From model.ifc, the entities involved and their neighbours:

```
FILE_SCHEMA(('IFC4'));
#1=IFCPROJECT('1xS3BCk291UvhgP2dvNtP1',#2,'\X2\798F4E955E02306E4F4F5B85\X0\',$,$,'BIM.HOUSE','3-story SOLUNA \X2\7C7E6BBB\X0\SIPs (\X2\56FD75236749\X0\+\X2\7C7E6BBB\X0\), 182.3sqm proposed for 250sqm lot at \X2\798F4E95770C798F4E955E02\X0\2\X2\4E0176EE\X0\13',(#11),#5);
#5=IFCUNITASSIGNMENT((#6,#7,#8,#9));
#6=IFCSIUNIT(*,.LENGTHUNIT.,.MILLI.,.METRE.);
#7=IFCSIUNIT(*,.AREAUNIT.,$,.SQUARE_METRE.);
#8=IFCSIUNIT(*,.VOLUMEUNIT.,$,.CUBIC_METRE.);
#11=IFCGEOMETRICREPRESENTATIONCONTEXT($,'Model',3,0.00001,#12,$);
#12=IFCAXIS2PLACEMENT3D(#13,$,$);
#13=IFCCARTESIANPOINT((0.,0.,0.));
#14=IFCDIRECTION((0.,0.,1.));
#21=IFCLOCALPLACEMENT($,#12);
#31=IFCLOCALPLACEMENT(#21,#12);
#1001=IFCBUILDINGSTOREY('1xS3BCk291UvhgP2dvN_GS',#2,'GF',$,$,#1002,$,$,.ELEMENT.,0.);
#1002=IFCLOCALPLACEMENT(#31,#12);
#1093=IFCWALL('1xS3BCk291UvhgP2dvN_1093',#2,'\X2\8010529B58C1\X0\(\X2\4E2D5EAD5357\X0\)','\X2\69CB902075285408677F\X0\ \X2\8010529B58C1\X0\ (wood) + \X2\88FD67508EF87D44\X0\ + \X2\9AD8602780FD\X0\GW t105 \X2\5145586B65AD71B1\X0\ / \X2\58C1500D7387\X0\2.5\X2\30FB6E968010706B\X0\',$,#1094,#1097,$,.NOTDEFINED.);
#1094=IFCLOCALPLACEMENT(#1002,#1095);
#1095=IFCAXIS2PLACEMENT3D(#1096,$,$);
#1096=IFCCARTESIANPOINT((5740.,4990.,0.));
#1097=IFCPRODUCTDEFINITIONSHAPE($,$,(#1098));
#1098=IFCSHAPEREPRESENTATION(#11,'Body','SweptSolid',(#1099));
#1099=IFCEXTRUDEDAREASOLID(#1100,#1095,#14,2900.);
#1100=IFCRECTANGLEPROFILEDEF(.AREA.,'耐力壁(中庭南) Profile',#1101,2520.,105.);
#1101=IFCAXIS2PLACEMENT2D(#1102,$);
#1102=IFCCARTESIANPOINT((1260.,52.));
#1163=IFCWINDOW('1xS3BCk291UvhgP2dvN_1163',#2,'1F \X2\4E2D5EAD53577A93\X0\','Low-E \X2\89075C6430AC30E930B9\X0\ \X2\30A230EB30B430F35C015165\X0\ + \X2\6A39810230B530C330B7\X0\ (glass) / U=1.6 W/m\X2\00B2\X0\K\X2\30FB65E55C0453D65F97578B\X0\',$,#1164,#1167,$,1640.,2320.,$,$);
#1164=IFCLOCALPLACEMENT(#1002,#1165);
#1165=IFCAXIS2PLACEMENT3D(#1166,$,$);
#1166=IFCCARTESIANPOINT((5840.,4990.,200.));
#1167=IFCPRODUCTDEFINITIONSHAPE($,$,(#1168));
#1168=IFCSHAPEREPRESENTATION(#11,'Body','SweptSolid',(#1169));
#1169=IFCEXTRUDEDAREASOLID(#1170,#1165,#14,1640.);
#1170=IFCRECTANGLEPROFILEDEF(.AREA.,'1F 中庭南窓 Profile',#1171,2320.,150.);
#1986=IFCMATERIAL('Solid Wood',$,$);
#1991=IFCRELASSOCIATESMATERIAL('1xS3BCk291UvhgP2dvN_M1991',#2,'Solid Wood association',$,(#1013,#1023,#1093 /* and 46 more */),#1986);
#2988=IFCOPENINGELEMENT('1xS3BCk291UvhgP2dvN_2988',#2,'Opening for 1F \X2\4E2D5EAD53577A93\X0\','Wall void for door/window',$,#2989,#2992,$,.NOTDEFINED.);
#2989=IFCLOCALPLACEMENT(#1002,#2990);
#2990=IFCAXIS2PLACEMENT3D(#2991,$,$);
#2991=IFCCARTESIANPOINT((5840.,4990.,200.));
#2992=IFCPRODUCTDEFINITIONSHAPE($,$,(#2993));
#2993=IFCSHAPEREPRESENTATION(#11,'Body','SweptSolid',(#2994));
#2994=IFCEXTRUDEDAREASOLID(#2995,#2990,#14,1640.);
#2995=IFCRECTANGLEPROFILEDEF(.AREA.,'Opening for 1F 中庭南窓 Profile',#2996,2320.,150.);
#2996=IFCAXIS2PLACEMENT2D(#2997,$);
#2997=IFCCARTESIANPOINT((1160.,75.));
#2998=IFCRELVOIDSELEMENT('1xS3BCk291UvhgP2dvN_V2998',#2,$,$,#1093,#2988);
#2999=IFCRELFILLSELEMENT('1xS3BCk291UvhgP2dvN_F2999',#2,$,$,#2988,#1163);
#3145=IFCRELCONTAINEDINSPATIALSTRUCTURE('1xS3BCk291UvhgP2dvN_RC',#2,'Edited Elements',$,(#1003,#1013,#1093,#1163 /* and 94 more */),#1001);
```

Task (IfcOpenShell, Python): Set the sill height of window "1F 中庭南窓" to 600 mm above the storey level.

```python
import numpy as np
import ifcopenshell
import ifcopenshell.api.geometry
import ifcopenshell.geom
import ifcopenshell.util.element
import ifcopenshell.util.placement
import ifcopenshell.util.shape
import ifcopenshell.util.unit

model = ifcopenshell.open("model.ifc")
unit_scale = ifcopenshell.util.unit.calculate_unit_scale(model)

window = model.by_id(1163)
opening = window.FillsVoids[0].RelatingOpeningElement
storey = ifcopenshell.util.element.get_container(window, ifc_class="IfcBuildingStorey")
level = ifcopenshell.util.placement.get_local_placement(storey.ObjectPlacement)[2, 3]

# The opening's origin need not be at the sill, so measure its lowest point.
shape = ifcopenshell.geom.create_shape(ifcopenshell.geom.settings(), opening)
bottom = ifcopenshell.util.shape.get_shape_bottom_elevation(shape, shape.geometry) / unit_scale
dz = level + 600.0 - bottom

shift = np.array([0.0, 0.0, dz])
# The window is not placed relative to its opening, so move both.
for product in (opening, window):
    matrix = ifcopenshell.util.placement.get_local_placement(product.ObjectPlacement)
    matrix[:3, 3] += shift
    ifcopenshell.api.geometry.edit_object_placement(model, product=product, matrix=matrix, is_si=False)

print(f"moved by {dz * unit_scale:+.3f} m")

model.write("model_v2.ifc")
```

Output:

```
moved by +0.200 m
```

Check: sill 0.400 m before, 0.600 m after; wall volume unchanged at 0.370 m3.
